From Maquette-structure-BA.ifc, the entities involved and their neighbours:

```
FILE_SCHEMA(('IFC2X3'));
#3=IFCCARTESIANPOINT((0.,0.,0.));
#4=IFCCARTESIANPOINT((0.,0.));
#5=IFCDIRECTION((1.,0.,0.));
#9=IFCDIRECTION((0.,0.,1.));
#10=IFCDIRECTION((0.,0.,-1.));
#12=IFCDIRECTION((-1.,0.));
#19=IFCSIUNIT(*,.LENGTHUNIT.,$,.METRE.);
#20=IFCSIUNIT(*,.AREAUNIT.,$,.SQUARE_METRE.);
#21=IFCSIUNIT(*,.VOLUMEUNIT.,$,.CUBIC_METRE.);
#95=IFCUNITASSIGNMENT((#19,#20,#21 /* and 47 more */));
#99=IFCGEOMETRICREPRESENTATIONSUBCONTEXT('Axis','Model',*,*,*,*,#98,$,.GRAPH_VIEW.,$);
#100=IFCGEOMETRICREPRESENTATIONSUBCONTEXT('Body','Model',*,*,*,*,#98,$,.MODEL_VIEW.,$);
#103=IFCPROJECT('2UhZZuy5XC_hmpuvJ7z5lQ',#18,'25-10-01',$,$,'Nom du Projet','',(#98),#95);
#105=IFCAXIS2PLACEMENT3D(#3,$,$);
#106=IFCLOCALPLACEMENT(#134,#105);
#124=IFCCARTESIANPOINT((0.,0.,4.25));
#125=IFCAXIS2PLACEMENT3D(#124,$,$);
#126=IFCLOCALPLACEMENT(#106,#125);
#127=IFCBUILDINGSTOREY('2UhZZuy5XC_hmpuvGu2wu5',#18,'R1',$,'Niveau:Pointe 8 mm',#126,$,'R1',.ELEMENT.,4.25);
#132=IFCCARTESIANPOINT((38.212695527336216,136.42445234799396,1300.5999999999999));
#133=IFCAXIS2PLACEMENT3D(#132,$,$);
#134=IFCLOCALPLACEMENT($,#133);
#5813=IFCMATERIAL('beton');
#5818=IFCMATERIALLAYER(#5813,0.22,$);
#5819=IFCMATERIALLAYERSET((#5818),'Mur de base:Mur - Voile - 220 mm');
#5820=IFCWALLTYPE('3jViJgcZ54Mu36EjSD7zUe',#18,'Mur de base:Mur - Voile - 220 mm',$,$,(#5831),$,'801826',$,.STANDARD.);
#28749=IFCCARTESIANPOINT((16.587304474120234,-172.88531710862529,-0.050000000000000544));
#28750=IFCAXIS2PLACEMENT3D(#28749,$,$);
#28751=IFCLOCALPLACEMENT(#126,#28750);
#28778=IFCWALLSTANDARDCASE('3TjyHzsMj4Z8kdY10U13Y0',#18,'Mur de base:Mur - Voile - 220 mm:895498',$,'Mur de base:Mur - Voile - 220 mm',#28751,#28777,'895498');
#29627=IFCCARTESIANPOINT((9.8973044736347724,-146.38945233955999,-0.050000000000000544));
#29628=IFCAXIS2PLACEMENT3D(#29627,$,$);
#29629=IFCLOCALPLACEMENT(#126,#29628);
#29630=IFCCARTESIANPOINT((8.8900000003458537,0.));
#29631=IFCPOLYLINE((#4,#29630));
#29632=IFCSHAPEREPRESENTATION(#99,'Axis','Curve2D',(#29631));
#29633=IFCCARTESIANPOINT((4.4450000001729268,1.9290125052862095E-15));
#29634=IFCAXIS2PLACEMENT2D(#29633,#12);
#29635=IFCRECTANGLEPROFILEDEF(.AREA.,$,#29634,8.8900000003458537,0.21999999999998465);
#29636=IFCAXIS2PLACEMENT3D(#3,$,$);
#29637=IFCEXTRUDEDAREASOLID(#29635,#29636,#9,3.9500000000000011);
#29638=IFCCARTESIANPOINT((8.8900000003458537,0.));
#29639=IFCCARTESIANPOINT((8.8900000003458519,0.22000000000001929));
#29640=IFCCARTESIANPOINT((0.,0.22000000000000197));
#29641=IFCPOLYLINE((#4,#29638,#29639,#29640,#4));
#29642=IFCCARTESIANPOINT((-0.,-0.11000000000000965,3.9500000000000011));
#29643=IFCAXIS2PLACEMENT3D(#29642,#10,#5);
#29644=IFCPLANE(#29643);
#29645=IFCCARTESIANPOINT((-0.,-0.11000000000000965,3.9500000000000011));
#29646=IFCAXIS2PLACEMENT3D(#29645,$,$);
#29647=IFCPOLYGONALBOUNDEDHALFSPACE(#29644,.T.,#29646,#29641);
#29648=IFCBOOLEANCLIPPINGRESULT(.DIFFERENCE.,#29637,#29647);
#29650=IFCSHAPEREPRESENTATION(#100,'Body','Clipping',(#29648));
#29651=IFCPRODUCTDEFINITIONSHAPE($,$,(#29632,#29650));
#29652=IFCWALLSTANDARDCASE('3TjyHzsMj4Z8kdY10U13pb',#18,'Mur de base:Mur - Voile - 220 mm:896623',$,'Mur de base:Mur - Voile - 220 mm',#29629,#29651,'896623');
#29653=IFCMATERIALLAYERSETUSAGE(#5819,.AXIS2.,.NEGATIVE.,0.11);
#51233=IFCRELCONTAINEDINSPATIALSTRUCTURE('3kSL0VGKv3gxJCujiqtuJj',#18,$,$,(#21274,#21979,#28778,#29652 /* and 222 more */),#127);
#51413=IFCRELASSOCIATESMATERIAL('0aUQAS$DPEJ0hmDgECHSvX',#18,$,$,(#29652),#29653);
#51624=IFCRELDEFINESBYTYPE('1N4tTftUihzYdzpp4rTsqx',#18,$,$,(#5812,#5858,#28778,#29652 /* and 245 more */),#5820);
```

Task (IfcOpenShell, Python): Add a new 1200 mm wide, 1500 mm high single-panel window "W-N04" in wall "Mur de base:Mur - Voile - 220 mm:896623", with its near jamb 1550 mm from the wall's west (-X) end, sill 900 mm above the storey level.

```python
import numpy as np
import ifcopenshell
import ifcopenshell.api.feature
import ifcopenshell.api.geometry
import ifcopenshell.api.root
import ifcopenshell.api.spatial
import ifcopenshell.api.type
import ifcopenshell.geom
import ifcopenshell.util.element
import ifcopenshell.util.placement
import ifcopenshell.util.representation
import ifcopenshell.util.shape
import ifcopenshell.util.unit

model = ifcopenshell.open("Maquette-structure-BA.ifc")
unit_scale = ifcopenshell.util.unit.calculate_unit_scale(model)
settings = ifcopenshell.geom.settings()


def volume(element):
    """Net volume in cubic metres, openings subtracted."""
    shape = ifcopenshell.geom.create_shape(settings, element)
    return ifcopenshell.util.shape.get_volume(shape.geometry)


wall = model.by_guid("3TjyHzsMj4Z8kdY10U13pb")
storey = ifcopenshell.util.element.get_container(wall, ifc_class="IfcBuildingStorey")
context = ifcopenshell.util.representation.get_context(model, "Model", "Body", "MODEL_VIEW")
before = volume(wall)

width, height, from_end, sill = 1.2, 1.5, 1.55, 0.9  # metres

# The wall runs along its own X axis, and the end named is its -X end.
wall_shape = ifcopenshell.geom.create_shape(settings, wall)
x, y, z = ifcopenshell.util.shape.get_vertices(wall_shape.geometry).T
start = x.min() + from_end
face, thickness = float(y.min()), float(y.max() - y.min())
wall_matrix = ifcopenshell.util.placement.get_local_placement(wall.ObjectPlacement)
level = ifcopenshell.util.placement.get_local_placement(storey.ObjectPlacement)[2, 3]


def in_wall(x, y):
    """Placement at x, y metres in the wall's axes, at sill height."""
    matrix = wall_matrix.copy()
    matrix[:, 3] = wall_matrix @ np.array([x / unit_scale, y / unit_scale, 0.0, 1.0])
    matrix[2, 3] = level + sill / unit_scale
    return matrix


# Opening: a box that overshoots both wall faces by 50 mm.
opening = ifcopenshell.api.root.create_entity(model, ifc_class="IfcOpeningElement")
box = ifcopenshell.api.geometry.add_wall_representation(
    model, context=context, length=width, height=height, thickness=thickness + 0.1
)
ifcopenshell.api.geometry.assign_representation(model, product=opening, representation=box)
ifcopenshell.api.geometry.edit_object_placement(model, product=opening, matrix=in_wall(start, face - 0.05), is_si=False)
ifcopenshell.api.feature.add_feature(model, feature=opening, element=wall)

window = ifcopenshell.api.root.create_entity(model, ifc_class="IfcWindow", name="W-N04")
window.OverallWidth, window.OverallHeight = width / unit_scale, height / unit_scale
body = ifcopenshell.api.geometry.add_window_representation(
    model,
    context=context,
    overall_width=window.OverallWidth,
    overall_height=window.OverallHeight,
    partition_type="SINGLE_PANEL",
)
ifcopenshell.api.geometry.assign_representation(model, product=window, representation=body)
ifcopenshell.api.spatial.assign_container(model, products=[window], relating_structure=storey)
fills = ifcopenshell.api.feature.add_filling(model, opening=opening, element=window)
fills.OwnerHistory = window.OwnerHistory  # required in IFC2X3

# IFC2X3 keeps the operation on the window style.
style = ifcopenshell.api.root.create_entity(model, ifc_class="IfcWindowStyle", name="W-N04")
style.OperationType, style.ConstructionType = "SINGLE_PANEL", "NOTDEFINED"
style.ParameterTakesPrecedence = style.Sizeable = False
ifcopenshell.api.type.assign_type(model, related_objects=[window], relating_type=style)

# Centre the window in the wall's thickness.
ifcopenshell.api.geometry.edit_object_placement(model, product=window, matrix=in_wall(start, face), is_si=False)
window_shape = ifcopenshell.geom.create_shape(settings, window)
depth = ifcopenshell.util.shape.get_vertices(window_shape.geometry)[:, 1]
offset = face + thickness / 2 - (depth.min() + depth.max()) / 2
ifcopenshell.api.geometry.edit_object_placement(model, product=window, matrix=in_wall(start, offset), is_si=False)

after = volume(wall)

print(f"wall volume {before:.3f} -> {after:.3f} m3")

model.write("Maquette-structure-BA-out.ifc")
```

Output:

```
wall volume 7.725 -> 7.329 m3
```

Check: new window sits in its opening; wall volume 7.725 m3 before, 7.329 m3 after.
